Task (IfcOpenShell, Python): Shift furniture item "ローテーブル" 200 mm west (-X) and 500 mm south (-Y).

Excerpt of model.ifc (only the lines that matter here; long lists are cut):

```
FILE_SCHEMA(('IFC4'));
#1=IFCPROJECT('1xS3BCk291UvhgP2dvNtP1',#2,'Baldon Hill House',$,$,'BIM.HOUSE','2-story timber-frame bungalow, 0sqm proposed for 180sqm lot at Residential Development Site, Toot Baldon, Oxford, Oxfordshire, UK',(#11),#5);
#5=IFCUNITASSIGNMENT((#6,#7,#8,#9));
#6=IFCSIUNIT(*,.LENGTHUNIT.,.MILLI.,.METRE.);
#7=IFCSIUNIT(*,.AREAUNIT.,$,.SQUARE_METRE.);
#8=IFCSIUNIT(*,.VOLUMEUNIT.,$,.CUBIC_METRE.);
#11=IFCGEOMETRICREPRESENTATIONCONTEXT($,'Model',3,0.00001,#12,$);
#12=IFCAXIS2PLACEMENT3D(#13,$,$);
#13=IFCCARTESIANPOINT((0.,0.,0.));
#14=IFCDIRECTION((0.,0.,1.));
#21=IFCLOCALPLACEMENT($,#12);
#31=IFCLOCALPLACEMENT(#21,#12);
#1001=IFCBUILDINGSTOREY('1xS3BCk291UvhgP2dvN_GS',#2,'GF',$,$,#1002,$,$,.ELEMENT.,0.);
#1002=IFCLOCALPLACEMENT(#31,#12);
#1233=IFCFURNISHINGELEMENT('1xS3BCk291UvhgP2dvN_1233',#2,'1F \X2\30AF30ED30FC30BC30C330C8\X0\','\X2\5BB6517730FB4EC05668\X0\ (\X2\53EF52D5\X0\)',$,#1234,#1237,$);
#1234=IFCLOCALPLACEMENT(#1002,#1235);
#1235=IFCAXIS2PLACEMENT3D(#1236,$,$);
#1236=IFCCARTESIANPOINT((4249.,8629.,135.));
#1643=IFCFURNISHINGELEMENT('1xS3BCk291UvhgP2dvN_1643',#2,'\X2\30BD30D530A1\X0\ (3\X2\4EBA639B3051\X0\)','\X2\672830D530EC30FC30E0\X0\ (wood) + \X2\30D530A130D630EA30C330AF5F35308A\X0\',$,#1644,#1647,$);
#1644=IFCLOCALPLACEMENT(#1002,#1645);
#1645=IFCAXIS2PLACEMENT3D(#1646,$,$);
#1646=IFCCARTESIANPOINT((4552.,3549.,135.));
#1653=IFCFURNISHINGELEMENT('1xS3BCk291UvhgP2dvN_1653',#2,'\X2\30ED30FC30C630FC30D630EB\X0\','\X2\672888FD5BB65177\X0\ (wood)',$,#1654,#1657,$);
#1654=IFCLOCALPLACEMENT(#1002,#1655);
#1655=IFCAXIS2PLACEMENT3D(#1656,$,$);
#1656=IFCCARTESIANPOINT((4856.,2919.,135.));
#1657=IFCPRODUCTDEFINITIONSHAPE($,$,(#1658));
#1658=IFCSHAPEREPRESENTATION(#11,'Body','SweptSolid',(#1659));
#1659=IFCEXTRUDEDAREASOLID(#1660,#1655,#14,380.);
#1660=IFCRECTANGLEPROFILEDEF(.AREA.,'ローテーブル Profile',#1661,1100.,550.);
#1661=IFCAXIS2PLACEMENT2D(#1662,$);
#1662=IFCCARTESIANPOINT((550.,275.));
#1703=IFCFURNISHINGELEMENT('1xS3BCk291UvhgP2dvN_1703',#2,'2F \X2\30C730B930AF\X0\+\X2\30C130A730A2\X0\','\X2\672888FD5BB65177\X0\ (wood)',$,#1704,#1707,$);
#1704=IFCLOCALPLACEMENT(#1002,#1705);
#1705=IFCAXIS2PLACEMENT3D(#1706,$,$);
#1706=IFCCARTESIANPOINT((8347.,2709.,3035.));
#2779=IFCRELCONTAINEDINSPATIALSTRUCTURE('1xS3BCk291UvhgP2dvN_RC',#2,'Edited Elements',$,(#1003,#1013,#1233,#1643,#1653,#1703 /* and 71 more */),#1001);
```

```python
import ifcopenshell
import ifcopenshell.api.geometry
import ifcopenshell.util.placement
import ifcopenshell.util.unit

model = ifcopenshell.open("model.ifc")
unit_scale = ifcopenshell.util.unit.calculate_unit_scale(model)

item = model.by_guid("1xS3BCk291UvhgP2dvN_1653")
matrix = ifcopenshell.util.placement.get_local_placement(item.ObjectPlacement)
matrix[0, 3] -= 0.2 / unit_scale
matrix[1, 3] -= 0.5 / unit_scale
ifcopenshell.api.geometry.edit_object_placement(model, product=item, matrix=matrix, is_si=False)

print(ifcopenshell.util.placement.get_local_placement(item.ObjectPlacement).round(3) + 0.0)

model.write("model_edited.ifc")
```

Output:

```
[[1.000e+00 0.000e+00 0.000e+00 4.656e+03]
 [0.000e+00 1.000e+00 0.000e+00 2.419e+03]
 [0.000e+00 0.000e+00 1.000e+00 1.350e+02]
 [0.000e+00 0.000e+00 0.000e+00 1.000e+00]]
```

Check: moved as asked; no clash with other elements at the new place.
